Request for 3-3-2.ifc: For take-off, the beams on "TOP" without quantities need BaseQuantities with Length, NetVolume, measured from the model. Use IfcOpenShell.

First a look at what the model holds.

```python
import ifcopenshell
import ifcopenshell.util.element
import ifcopenshell.util.unit

model = ifcopenshell.open("3-3-2.ifc")
print(model.schema)
for unit_type in ("LENGTHUNIT", "AREAUNIT", "VOLUMEUNIT"):
    print(unit_type, ifcopenshell.util.unit.calculate_unit_scale(model, unit_type))
storey = next(s for s in model.by_type("IfcBuildingStorey") if s.Name == "TOP")
beams = [e for e in ifcopenshell.util.element.get_decomposition(storey) if e.is_a("IfcBeam")]
for e in sorted(beams, key=lambda e: e.id()):
    print(e.id(), e.is_a(), e.Name, list(ifcopenshell.util.element.get_psets(e, qtos_only=True)), sep=" | ")
```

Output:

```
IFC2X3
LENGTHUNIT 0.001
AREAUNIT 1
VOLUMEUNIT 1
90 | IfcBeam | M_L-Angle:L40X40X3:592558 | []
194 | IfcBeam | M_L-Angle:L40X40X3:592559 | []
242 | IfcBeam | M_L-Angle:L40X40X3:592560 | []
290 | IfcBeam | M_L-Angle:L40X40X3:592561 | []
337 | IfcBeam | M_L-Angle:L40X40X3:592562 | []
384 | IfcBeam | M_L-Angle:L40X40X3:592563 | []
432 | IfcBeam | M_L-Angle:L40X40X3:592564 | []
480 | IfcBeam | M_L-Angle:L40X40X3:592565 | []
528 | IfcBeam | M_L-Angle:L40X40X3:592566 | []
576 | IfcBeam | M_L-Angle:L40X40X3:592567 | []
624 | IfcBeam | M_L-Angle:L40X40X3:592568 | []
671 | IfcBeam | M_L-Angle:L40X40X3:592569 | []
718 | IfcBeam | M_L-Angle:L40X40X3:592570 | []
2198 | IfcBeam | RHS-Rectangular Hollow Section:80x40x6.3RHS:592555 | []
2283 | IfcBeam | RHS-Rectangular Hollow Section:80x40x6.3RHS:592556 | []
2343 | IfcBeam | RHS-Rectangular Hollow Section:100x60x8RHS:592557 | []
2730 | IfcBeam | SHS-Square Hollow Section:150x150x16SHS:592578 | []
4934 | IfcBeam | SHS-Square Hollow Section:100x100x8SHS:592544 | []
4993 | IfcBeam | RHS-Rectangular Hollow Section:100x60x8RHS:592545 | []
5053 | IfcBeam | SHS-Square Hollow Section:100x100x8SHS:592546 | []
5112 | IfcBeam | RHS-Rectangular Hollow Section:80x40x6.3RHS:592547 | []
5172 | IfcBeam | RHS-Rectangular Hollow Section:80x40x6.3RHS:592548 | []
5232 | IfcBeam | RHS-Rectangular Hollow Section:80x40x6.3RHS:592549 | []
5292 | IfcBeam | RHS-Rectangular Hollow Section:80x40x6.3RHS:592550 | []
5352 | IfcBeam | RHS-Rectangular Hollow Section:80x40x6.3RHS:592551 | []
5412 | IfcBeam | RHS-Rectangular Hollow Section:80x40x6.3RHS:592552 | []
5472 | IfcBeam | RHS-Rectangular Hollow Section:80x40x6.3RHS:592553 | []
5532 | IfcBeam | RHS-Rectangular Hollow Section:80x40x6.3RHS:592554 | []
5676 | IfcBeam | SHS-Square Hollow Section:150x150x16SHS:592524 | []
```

```python
import ifcopenshell
import ifcopenshell.api.pset
import ifcopenshell.geom
import ifcopenshell.util.element
import ifcopenshell.util.shape
import ifcopenshell.util.unit

model = ifcopenshell.open("3-3-2.ifc")
unit_scale = ifcopenshell.util.unit.calculate_unit_scale(model)
volume_scale = ifcopenshell.util.unit.calculate_unit_scale(model, "VOLUMEUNIT")
settings = ifcopenshell.geom.settings()

storey = next(s for s in model.by_type("IfcBuildingStorey") if s.Name == "TOP")
beams = [e for e in ifcopenshell.util.element.get_decomposition(storey) if e.is_a("IfcBeam")]

for e in sorted(beams, key=lambda e: e.id()):
    if ifcopenshell.util.element.get_psets(e, qtos_only=True, should_inherit=False):
        continue
    # Geometry comes back in metres, in the element's own axes.
    shape = ifcopenshell.geom.create_shape(settings, e)
    values = {
        "Length": ifcopenshell.util.shape.get_max_xyz(shape.geometry) / unit_scale,
        "NetVolume": ifcopenshell.util.shape.get_volume(shape.geometry) / volume_scale,
    }
    qto = ifcopenshell.api.pset.add_qto(model, product=e, name="BaseQuantities")
    ifcopenshell.api.pset.edit_qto(model, qto=qto, properties=values)
    print(e.id(), {k: round(v, 3) for k, v in values.items()})

model.write("3-3-2_edited.ifc")
```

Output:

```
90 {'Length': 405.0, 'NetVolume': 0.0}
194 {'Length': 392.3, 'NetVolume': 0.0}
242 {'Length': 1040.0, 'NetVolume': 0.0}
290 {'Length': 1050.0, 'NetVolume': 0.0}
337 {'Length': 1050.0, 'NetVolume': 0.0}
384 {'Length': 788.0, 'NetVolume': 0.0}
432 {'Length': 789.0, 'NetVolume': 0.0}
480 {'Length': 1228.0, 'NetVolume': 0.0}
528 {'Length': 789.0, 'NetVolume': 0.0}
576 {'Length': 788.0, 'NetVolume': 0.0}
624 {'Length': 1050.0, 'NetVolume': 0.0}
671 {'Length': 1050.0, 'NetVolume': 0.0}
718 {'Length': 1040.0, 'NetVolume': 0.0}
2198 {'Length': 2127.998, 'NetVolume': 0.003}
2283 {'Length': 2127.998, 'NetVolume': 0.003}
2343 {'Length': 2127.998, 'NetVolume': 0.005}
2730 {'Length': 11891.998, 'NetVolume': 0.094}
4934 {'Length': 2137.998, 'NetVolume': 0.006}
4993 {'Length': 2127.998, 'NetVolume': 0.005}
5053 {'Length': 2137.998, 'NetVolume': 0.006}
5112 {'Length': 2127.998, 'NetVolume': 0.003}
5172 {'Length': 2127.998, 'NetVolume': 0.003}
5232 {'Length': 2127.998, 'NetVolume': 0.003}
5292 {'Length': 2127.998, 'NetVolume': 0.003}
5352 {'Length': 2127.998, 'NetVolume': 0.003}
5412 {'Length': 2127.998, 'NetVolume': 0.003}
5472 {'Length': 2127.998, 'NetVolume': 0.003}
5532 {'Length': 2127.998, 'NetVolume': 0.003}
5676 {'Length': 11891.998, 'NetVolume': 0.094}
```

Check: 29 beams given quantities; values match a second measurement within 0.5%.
